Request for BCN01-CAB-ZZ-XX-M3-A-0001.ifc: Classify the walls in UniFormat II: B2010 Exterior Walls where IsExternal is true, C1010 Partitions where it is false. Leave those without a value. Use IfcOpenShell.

First a look at what the model holds.

```python
import ifcopenshell
import ifcopenshell.util.element

model = ifcopenshell.open("BCN01-CAB-ZZ-XX-M3-A-0001.ifc")
print(model.schema)
print("classifications:", [c.Name for c in model.by_type("IfcClassification")])
values = [ifcopenshell.util.element.get_pset(e, "Pset_WallCommon", "IsExternal") for e in model.by_type("IfcWall")]
for value in (True, False, None):
    print("IsExternal", value, values.count(value))
```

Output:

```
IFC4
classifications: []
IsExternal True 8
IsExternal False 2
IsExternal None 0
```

```python
import ifcopenshell
import ifcopenshell.api.classification
import ifcopenshell.util.element

model = ifcopenshell.open("BCN01-CAB-ZZ-XX-M3-A-0001.ifc")

system = ifcopenshell.api.classification.add_classification(model, classification="UniFormat II")

walls = model.by_type("IfcWall")
external = {e: ifcopenshell.util.element.get_pset(e, "Pset_WallCommon", "IsExternal") for e in walls}
for flag, code, name in ((True, "B2010", "Exterior Walls"), (False, "C1010", "Partitions")):
    products = [e for e in walls if external[e] is flag]
    ifcopenshell.api.classification.add_reference(
        model, products=products, classification=system, identification=code, name=name
    )
    print(code, len(products))

model.write("BCN01-CAB-ZZ-XX-M3-A-0001-out.ifc")
```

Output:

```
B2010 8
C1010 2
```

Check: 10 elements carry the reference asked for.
